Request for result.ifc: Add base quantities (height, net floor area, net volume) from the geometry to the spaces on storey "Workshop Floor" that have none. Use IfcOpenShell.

First a look at what the model holds.

```python
import ifcopenshell
import ifcopenshell.util.element
import ifcopenshell.util.unit

model = ifcopenshell.open("result.ifc")
print(model.schema)
for unit_type in ("LENGTHUNIT", "AREAUNIT", "VOLUMEUNIT"):
    print(unit_type, ifcopenshell.util.unit.calculate_unit_scale(model, unit_type))
storey = next(s for s in model.by_type("IfcBuildingStorey") if s.Name == "Workshop Floor")
spaces = [e for e in ifcopenshell.util.element.get_decomposition(storey) if e.is_a("IfcSpace")]
for e in sorted(spaces, key=lambda e: e.id()):
    print(e.id(), e.is_a(), e.Name, list(ifcopenshell.util.element.get_psets(e, qtos_only=True)), sep=" | ")
```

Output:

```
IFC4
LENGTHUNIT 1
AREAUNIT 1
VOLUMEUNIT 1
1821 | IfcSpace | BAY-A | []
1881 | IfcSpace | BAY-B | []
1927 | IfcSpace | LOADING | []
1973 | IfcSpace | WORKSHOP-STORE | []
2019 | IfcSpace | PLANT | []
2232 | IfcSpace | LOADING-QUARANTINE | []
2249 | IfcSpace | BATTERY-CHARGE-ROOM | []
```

```python
import ifcopenshell
import ifcopenshell.api.pset
import ifcopenshell.geom
import ifcopenshell.util.element
import ifcopenshell.util.shape
import ifcopenshell.util.unit

model = ifcopenshell.open("result.ifc")
unit_scale = ifcopenshell.util.unit.calculate_unit_scale(model)
area_scale = ifcopenshell.util.unit.calculate_unit_scale(model, "AREAUNIT")
volume_scale = ifcopenshell.util.unit.calculate_unit_scale(model, "VOLUMEUNIT")
settings = ifcopenshell.geom.settings()

storey = next(s for s in model.by_type("IfcBuildingStorey") if s.Name == "Workshop Floor")
spaces = [e for e in ifcopenshell.util.element.get_decomposition(storey) if e.is_a("IfcSpace")]

for e in sorted(spaces, key=lambda e: e.id()):
    if ifcopenshell.util.element.get_psets(e, qtos_only=True, should_inherit=False):
        continue
    # Geometry comes back in metres, in the element's own axes.
    shape = ifcopenshell.geom.create_shape(settings, e)
    values = {
        "Height": ifcopenshell.util.shape.get_z(shape.geometry) / unit_scale,
        "NetFloorArea": ifcopenshell.util.shape.get_footprint_area(shape.geometry) / area_scale,
        "NetVolume": ifcopenshell.util.shape.get_volume(shape.geometry) / volume_scale,
    }
    qto = ifcopenshell.api.pset.add_qto(model, product=e, name="Qto_SpaceBaseQuantities")
    ifcopenshell.api.pset.edit_qto(model, qto=qto, properties=values)
    print(e.id(), {k: round(v, 3) for k, v in values.items()})

model.write("result_updated.ifc")
```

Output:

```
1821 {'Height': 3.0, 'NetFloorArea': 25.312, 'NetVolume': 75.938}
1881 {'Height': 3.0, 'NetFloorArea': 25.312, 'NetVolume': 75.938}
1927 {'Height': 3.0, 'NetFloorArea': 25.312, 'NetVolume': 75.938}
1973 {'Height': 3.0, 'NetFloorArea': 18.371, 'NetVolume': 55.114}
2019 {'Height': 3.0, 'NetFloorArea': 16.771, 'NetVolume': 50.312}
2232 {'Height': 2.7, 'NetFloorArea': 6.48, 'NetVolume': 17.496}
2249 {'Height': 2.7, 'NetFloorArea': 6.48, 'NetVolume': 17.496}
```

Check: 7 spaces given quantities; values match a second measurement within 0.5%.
